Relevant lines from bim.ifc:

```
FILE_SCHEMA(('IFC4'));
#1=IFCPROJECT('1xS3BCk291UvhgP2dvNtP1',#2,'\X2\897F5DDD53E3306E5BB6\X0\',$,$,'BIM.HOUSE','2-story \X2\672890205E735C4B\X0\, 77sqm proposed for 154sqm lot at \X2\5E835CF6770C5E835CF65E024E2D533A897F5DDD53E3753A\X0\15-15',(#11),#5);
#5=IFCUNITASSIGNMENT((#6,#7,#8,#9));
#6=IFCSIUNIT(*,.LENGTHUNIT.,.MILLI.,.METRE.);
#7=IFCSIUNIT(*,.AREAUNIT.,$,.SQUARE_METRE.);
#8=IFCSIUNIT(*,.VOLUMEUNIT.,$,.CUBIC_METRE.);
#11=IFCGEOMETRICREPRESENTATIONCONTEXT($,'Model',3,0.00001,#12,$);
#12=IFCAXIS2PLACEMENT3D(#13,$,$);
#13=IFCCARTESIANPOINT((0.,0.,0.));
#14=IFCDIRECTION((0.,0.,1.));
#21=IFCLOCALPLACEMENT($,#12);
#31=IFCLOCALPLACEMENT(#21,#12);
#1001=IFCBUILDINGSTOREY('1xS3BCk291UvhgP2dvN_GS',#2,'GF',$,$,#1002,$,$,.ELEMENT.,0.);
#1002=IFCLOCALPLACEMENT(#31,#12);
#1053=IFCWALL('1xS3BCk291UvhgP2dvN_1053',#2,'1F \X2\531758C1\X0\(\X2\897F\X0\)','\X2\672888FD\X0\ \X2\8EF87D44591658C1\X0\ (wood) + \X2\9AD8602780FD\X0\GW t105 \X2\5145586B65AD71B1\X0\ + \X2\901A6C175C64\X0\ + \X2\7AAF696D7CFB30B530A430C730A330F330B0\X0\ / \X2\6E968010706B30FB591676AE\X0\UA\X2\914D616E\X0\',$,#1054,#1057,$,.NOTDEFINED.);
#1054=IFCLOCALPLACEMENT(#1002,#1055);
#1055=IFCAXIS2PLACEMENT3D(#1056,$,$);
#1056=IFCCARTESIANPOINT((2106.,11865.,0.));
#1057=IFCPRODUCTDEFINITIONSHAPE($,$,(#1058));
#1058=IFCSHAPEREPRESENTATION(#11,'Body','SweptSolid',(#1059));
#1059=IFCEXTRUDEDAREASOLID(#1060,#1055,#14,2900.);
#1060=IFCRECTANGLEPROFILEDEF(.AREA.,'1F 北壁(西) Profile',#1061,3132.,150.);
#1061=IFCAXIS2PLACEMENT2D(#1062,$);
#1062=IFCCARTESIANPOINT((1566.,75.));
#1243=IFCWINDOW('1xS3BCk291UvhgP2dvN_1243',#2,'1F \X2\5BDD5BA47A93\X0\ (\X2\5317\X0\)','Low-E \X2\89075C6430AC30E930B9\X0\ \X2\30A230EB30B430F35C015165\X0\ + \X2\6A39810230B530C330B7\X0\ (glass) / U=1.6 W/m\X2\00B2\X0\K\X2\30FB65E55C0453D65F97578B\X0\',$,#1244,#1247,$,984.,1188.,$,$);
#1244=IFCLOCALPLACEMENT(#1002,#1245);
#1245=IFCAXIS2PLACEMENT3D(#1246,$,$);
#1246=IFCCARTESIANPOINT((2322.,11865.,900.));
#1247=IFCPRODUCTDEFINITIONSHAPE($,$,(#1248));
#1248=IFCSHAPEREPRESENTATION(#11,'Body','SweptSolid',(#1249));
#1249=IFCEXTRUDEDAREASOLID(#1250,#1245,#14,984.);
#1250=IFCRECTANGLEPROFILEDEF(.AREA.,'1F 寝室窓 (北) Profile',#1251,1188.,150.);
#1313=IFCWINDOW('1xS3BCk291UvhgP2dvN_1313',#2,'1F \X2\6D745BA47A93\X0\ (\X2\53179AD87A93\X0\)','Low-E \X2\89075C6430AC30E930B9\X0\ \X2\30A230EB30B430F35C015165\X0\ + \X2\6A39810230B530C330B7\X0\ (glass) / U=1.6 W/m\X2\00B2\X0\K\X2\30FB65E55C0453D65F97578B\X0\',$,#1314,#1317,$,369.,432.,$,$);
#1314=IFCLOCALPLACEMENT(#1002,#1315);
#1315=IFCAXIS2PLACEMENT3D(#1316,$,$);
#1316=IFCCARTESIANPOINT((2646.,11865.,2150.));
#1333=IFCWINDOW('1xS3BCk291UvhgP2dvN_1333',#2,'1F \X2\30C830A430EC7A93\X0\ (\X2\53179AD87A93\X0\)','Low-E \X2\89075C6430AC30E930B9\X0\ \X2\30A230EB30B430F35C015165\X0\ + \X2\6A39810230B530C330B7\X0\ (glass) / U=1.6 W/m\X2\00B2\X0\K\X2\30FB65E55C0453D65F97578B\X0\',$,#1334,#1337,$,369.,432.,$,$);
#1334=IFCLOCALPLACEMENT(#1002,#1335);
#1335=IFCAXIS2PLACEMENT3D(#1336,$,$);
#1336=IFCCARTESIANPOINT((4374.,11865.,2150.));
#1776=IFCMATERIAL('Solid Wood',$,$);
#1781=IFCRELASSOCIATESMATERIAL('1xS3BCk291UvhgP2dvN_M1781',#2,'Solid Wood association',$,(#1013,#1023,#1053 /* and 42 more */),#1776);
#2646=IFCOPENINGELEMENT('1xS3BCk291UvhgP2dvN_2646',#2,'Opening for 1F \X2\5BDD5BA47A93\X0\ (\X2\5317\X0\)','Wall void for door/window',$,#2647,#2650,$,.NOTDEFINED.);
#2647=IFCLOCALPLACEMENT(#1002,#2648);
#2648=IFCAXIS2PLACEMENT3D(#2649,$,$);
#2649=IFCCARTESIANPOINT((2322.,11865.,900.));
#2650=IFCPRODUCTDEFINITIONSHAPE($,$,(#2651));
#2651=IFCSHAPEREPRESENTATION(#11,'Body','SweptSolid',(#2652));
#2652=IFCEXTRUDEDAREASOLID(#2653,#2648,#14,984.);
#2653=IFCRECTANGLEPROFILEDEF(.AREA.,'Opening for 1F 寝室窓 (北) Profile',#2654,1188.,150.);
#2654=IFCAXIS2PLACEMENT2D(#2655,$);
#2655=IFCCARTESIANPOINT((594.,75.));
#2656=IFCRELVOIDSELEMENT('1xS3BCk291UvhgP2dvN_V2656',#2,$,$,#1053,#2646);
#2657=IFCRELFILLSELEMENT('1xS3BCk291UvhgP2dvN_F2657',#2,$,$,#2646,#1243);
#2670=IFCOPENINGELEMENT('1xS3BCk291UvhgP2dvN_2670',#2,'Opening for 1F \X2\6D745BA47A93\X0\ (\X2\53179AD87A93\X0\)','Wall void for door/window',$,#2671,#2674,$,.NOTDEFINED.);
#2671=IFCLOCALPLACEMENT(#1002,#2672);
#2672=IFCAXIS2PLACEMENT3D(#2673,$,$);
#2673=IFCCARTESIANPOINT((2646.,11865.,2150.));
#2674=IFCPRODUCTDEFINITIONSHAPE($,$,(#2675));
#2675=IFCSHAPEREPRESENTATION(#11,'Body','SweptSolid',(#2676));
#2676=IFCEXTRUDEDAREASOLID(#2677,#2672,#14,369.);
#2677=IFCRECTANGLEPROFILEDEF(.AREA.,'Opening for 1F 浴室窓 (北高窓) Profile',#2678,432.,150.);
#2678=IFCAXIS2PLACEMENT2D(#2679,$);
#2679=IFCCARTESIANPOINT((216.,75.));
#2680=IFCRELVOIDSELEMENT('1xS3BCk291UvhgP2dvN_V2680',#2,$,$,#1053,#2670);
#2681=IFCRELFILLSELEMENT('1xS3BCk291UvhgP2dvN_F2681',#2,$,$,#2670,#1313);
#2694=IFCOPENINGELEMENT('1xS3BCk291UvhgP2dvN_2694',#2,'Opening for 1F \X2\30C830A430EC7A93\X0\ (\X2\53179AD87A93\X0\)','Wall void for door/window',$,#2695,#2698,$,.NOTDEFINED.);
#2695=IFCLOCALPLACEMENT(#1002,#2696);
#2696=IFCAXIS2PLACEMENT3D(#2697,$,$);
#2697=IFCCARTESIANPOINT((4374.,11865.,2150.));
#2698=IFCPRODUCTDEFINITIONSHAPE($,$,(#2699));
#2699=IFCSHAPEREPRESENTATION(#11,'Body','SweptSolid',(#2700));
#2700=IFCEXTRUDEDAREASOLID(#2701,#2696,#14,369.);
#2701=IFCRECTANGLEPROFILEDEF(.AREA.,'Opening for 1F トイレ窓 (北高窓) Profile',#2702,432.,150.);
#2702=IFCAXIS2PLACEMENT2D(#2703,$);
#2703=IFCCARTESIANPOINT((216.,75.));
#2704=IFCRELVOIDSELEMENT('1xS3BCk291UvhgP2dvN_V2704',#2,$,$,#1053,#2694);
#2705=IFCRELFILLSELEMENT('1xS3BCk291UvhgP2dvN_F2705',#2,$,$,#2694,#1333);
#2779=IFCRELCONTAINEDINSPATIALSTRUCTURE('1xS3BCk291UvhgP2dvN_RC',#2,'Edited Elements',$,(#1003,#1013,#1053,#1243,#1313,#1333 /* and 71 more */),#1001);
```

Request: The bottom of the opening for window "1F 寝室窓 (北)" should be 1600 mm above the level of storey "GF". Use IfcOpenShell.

```python
import numpy as np
import ifcopenshell
import ifcopenshell.api.geometry
import ifcopenshell.geom
import ifcopenshell.util.element
import ifcopenshell.util.placement
import ifcopenshell.util.shape
import ifcopenshell.util.unit

model = ifcopenshell.open("bim.ifc")
unit_scale = ifcopenshell.util.unit.calculate_unit_scale(model)

window = model.by_id(1243)
opening = window.FillsVoids[0].RelatingOpeningElement
storey = ifcopenshell.util.element.get_container(window, ifc_class="IfcBuildingStorey")
level = ifcopenshell.util.placement.get_local_placement(storey.ObjectPlacement)[2, 3]

# The opening's origin need not be at the sill, so measure its lowest point.
shape = ifcopenshell.geom.create_shape(ifcopenshell.geom.settings(), opening)
bottom = ifcopenshell.util.shape.get_shape_bottom_elevation(shape, shape.geometry) / unit_scale
dz = level + 1600.0 - bottom

shift = np.array([0.0, 0.0, dz])
# The window is not placed relative to its opening, so move both.
for product in (opening, window):
    matrix = ifcopenshell.util.placement.get_local_placement(product.ObjectPlacement)
    matrix[:3, 3] += shift
    ifcopenshell.api.geometry.edit_object_placement(model, product=product, matrix=matrix, is_si=False)

print(f"moved by {dz * unit_scale:+.3f} m")

model.write("bim_updated.ifc")
```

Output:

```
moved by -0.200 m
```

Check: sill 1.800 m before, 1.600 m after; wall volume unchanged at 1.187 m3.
